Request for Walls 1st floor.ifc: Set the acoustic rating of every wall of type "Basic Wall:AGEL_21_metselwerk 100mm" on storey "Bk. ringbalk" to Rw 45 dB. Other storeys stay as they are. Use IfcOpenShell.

First a look at what the model holds.

```python
import ifcopenshell
import ifcopenshell.util.element

model = ifcopenshell.open("Walls 1st floor.ifc")
print(model.schema)
storey = next(s for s in model.by_type("IfcBuildingStorey") if s.Name == "Bk. ringbalk")
walls = [e for e in ifcopenshell.util.element.get_decomposition(storey) if e.is_a("IfcWall")]
seen = {}
for e in walls:
    element_type = ifcopenshell.util.element.get_type(e)
    key = (element_type.Name if element_type != e and element_type else None, ifcopenshell.util.element.get_pset(e, "Pset_WallCommon", "AcousticRating"))
    seen[key] = seen.get(key, 0) + 1
for (name, value), count in sorted(seen.items(), key=str):
    print(count, "x", name, "|", value)
```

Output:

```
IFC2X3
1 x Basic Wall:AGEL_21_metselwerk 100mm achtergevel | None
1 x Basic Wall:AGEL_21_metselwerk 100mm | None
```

```python
import ifcopenshell
import ifcopenshell.api.pset
import ifcopenshell.util.element

model = ifcopenshell.open("Walls 1st floor.ifc")

storey = next(s for s in model.by_type("IfcBuildingStorey") if s.Name == "Bk. ringbalk")
walls = [e for e in ifcopenshell.util.element.get_decomposition(storey) if e.is_a("IfcWall")]

count = 0
for e in walls:
    element_type = ifcopenshell.util.element.get_type(e)
    if element_type in (None, e) or element_type.Name != "Basic Wall:AGEL_21_metselwerk 100mm":
        continue
    # add_pset returns the element's existing set when there is one.
    pset = ifcopenshell.api.pset.add_pset(model, product=e, name="Pset_WallCommon")
    ifcopenshell.api.pset.edit_pset(model, pset=pset, properties={"AcousticRating": "Rw 45 dB"})
    count += 1

print(count, "walls updated")

model.write("Walls 1st floor_edited.ifc")
```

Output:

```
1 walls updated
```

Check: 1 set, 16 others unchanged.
